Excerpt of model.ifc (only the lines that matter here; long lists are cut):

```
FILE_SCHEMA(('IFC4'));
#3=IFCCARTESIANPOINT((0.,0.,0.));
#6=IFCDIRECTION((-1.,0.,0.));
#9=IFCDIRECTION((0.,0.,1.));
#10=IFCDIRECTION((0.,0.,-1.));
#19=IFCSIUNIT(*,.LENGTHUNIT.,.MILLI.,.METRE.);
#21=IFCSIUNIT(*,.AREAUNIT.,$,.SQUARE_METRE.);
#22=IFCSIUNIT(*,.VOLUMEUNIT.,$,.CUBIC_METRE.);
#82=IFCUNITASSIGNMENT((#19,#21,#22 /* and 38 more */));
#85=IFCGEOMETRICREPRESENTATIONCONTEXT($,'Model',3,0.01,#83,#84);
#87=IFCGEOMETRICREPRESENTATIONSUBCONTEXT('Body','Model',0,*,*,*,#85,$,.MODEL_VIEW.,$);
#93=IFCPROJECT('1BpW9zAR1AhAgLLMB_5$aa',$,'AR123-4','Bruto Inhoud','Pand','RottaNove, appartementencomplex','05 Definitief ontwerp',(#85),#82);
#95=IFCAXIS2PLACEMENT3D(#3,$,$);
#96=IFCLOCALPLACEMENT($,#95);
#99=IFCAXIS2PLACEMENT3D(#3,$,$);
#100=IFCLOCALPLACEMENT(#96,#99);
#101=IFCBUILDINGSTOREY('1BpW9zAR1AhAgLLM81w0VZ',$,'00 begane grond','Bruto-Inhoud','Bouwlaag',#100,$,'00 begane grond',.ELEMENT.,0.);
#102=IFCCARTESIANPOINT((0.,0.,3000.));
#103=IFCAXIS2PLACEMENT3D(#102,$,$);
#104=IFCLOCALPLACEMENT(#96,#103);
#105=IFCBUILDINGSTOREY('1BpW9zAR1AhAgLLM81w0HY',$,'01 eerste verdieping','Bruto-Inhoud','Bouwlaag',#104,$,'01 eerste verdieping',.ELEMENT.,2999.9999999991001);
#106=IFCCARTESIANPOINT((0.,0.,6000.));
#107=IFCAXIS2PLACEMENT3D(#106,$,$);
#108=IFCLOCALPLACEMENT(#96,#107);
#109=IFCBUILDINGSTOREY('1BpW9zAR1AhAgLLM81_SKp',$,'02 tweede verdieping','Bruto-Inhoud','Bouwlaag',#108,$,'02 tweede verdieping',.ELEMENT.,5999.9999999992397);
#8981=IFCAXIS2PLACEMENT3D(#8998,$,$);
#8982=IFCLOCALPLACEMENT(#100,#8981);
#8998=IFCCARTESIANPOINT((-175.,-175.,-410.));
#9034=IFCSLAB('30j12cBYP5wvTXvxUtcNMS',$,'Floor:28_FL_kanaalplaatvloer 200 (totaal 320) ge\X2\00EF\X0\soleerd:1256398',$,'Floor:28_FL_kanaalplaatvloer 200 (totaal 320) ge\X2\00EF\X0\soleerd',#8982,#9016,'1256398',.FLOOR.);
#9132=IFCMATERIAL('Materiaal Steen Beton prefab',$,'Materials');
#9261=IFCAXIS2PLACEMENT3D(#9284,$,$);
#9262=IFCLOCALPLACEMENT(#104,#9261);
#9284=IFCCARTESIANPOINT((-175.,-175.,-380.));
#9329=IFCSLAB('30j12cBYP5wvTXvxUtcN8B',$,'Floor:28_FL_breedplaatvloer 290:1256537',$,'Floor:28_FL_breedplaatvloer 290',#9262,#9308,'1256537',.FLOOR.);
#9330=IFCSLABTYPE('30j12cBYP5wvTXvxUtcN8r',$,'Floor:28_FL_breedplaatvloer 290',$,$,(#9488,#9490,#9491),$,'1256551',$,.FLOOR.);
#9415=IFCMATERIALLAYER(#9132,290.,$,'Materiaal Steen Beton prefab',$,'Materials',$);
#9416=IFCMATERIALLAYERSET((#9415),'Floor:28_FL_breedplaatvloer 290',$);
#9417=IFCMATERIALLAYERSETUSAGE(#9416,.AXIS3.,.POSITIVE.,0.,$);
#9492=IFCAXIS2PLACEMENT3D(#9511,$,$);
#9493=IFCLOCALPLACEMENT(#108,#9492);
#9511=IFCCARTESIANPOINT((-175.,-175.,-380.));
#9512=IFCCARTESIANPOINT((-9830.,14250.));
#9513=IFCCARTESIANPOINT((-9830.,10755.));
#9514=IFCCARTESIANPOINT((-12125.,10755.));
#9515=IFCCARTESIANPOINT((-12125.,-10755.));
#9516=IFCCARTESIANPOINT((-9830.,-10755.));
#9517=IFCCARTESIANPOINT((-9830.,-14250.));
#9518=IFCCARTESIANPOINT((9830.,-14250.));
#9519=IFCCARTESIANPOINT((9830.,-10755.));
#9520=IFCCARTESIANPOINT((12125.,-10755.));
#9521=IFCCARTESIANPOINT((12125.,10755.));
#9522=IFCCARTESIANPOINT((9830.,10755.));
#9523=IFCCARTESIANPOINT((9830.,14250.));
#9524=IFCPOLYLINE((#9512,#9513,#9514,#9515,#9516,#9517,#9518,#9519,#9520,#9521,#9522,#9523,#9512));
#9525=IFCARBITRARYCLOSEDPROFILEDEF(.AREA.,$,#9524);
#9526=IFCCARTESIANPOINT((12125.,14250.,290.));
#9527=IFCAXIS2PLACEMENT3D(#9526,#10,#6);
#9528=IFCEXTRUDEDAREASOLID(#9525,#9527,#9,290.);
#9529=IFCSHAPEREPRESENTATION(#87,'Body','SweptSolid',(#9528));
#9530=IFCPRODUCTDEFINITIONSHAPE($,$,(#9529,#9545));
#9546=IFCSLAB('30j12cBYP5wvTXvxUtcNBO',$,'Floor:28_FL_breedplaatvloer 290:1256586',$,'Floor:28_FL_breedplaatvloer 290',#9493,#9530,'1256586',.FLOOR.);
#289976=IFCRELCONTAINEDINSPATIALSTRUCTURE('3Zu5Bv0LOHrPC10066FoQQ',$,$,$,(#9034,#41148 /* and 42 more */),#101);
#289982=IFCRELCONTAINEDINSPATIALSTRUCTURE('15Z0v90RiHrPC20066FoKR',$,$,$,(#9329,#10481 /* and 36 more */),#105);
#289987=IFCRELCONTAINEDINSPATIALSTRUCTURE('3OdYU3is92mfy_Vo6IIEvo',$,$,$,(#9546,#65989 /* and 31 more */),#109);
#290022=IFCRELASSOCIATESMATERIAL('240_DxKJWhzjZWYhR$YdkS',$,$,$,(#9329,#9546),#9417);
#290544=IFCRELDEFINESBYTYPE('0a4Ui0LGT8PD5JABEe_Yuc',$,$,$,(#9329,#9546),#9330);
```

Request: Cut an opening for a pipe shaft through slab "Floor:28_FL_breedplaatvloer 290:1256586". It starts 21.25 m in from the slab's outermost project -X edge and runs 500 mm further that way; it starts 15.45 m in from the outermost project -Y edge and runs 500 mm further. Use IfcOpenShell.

```python
import numpy as np
import ifcopenshell
import ifcopenshell.api.feature
import ifcopenshell.api.geometry
import ifcopenshell.api.root
import ifcopenshell.geom
import ifcopenshell.util.placement
import ifcopenshell.util.representation
import ifcopenshell.util.shape
import ifcopenshell.util.unit

model = ifcopenshell.open("model.ifc")
unit_scale = ifcopenshell.util.unit.calculate_unit_scale(model)
settings = ifcopenshell.geom.settings()


def volume(element):
    """Net volume in cubic metres, openings subtracted."""
    shape = ifcopenshell.geom.create_shape(settings, element)
    return ifcopenshell.util.shape.get_volume(shape.geometry)


slab = model.by_guid("30j12cBYP5wvTXvxUtcNBO")
before = volume(slab)

# Extent in the slab's own axes, in metres. The edges named are its -X and -Y sides.
slab_shape = ifcopenshell.geom.create_shape(settings, slab)
vertices = ifcopenshell.util.shape.get_vertices(slab_shape.geometry)
x_min, y_min, bottom = vertices.min(axis=0)
top = vertices[:, 2].max()

opening = ifcopenshell.api.root.create_entity(model, ifc_class="IfcOpeningElement", name="Pipe shaft opening", predefined_type="OPENING")
context = ifcopenshell.util.representation.get_context(model, "Model", "Body", "MODEL_VIEW")
width, depth = 0.5, 0.5
outline = [(0.0, 0.0), (width, 0.0), (width, depth), (0.0, depth), (0.0, 0.0)]
# Overshoot both faces by 50 mm so the cut is clean.
shape = ifcopenshell.api.geometry.add_slab_representation(
    model, context=context, depth=top - bottom + 0.1, polyline=outline
)
ifcopenshell.api.geometry.assign_representation(model, product=opening, representation=shape)

matrix = ifcopenshell.util.placement.get_local_placement(slab.ObjectPlacement)
matrix[:, 3] = matrix @ np.append(np.array([x_min + 21.25, y_min + 15.45, bottom - 0.05]) / unit_scale, 1.0)
ifcopenshell.api.geometry.edit_object_placement(model, product=opening, matrix=matrix, is_si=False)
ifcopenshell.api.feature.add_feature(model, feature=opening, element=slab)

after = volume(slab)

print(f"slab volume {before:.3f} -> {after:.3f} m3")

model.write("model_v2.ifc")
```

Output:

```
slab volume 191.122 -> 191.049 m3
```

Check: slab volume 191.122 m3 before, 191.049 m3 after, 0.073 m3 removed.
